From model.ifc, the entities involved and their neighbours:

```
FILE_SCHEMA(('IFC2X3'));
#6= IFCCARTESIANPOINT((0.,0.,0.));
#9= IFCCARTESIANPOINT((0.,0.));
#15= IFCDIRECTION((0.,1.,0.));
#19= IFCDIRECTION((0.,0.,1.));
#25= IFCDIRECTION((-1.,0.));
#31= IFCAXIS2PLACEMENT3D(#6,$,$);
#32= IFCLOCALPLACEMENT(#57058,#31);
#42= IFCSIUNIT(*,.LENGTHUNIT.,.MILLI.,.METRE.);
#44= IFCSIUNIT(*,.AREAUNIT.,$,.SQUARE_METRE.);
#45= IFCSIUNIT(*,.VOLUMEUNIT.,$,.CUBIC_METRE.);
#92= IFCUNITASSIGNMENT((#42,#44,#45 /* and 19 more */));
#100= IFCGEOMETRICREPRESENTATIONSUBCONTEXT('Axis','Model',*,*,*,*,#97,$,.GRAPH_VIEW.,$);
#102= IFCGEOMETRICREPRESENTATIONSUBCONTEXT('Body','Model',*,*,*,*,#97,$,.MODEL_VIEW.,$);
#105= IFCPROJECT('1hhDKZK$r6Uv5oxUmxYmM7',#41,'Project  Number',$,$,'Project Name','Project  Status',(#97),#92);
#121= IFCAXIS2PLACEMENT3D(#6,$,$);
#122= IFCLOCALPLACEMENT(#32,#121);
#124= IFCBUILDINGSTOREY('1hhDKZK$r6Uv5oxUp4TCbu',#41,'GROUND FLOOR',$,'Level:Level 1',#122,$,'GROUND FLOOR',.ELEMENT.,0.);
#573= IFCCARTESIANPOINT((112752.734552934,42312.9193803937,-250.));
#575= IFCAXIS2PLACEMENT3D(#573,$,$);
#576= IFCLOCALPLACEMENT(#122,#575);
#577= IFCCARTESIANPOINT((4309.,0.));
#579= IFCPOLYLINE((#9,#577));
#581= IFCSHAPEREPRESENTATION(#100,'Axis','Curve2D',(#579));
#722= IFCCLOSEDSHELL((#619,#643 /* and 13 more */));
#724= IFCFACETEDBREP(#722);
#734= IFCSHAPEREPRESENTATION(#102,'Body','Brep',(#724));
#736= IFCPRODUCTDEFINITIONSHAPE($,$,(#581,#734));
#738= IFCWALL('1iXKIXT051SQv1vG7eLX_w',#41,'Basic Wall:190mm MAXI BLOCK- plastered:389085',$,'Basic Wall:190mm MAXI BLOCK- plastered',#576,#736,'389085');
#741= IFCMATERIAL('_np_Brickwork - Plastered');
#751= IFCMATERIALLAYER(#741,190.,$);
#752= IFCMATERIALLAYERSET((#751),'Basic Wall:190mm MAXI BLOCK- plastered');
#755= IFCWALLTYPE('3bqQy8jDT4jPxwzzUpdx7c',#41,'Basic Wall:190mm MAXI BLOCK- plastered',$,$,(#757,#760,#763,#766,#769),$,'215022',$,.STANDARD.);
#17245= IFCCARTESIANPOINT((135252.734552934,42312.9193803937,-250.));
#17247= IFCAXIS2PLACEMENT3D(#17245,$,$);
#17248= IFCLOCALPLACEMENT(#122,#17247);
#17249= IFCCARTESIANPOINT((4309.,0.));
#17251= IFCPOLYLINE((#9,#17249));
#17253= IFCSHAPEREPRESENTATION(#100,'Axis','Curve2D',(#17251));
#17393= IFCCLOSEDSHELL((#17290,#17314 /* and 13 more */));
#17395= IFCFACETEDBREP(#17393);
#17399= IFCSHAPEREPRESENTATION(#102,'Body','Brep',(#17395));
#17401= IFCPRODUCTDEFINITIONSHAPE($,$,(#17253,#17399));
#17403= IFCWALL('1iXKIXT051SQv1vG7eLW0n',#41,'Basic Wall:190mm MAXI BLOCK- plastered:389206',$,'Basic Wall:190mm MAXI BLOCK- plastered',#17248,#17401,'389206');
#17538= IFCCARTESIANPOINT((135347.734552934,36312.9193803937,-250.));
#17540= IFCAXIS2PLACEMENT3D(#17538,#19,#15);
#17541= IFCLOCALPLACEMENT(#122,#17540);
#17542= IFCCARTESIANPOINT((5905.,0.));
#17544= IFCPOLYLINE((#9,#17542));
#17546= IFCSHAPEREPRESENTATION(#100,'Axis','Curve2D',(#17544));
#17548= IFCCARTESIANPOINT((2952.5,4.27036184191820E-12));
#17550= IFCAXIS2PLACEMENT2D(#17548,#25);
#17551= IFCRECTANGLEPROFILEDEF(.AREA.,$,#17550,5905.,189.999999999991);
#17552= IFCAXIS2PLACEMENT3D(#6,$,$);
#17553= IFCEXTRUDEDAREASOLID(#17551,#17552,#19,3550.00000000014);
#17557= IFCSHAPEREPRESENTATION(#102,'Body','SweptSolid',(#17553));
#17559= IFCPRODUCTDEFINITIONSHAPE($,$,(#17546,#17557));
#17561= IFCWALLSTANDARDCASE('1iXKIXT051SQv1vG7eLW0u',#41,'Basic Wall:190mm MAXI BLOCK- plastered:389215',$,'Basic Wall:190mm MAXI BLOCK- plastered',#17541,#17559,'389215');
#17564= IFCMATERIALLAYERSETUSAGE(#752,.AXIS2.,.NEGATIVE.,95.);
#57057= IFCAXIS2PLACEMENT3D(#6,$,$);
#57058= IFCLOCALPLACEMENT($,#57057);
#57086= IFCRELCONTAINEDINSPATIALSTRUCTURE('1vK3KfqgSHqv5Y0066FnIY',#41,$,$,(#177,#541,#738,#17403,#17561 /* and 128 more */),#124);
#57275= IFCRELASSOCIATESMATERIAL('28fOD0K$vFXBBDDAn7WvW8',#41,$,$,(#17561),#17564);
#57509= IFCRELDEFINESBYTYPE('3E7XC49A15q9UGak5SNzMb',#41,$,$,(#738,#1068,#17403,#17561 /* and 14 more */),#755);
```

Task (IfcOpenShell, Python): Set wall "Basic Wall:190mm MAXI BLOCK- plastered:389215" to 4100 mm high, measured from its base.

```python
import ifcopenshell
import ifcopenshell.geom
import ifcopenshell.util.representation
import ifcopenshell.util.shape
import ifcopenshell.util.unit

model = ifcopenshell.open("model.ifc")
unit_scale = ifcopenshell.util.unit.calculate_unit_scale(model)
settings = ifcopenshell.geom.settings()


def volume(element):
    """Net volume in cubic metres, openings subtracted."""
    shape = ifcopenshell.geom.create_shape(settings, element)
    return ifcopenshell.util.shape.get_volume(shape.geometry)


wall = model.by_guid("1iXKIXT051SQv1vG7eLW0u")
before = volume(wall)

body = ifcopenshell.util.representation.get_representation(wall, "Model", "Body")
solid = body.Items[0]
old_height = solid.Depth
solid.Depth = 4.1 / unit_scale
after = volume(wall)

print(f"height {old_height:g} -> {solid.Depth:g}, volume {before:.3f} -> {after:.3f} m3")

model.write("model_v2.ifc")
```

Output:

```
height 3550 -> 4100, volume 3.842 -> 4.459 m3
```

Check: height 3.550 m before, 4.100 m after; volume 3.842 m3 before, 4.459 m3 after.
